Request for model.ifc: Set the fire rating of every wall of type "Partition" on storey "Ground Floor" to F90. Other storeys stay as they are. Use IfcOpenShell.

First a look at what the model holds.

```python
import ifcopenshell
import ifcopenshell.util.element

model = ifcopenshell.open("model.ifc")
print(model.schema)
storey = next(s for s in model.by_type("IfcBuildingStorey") if s.Name == "Ground Floor")
walls = [e for e in ifcopenshell.util.element.get_decomposition(storey) if e.is_a("IfcWall")]
seen = {}
for e in walls:
    element_type = ifcopenshell.util.element.get_type(e)
    key = (element_type.Name if element_type != e and element_type else None, ifcopenshell.util.element.get_pset(e, "Pset_WallCommon", "FireRating"))
    seen[key] = seen.get(key, 0) + 1
for (name, value), count in sorted(seen.items(), key=str):
    print(count, "x", name, "|", value)
```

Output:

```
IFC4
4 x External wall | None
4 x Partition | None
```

```python
import ifcopenshell
import ifcopenshell.api.pset
import ifcopenshell.util.element

model = ifcopenshell.open("model.ifc")

storey = next(s for s in model.by_type("IfcBuildingStorey") if s.Name == "Ground Floor")
walls = [e for e in ifcopenshell.util.element.get_decomposition(storey) if e.is_a("IfcWall")]

count = 0
for e in walls:
    element_type = ifcopenshell.util.element.get_type(e)
    if element_type in (None, e) or element_type.Name != "Partition":
        continue
    # add_pset returns the element's existing set when there is one.
    pset = ifcopenshell.api.pset.add_pset(model, product=e, name="Pset_WallCommon")
    ifcopenshell.api.pset.edit_pset(model, pset=pset, properties={"FireRating": "F90"})
    count += 1

print(count, "walls updated")

model.write("model_updated.ifc")
```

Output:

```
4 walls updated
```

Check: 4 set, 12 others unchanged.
